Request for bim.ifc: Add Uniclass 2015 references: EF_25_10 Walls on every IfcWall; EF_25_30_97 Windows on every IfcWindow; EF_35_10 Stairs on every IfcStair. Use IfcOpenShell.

First a look at what the model holds.

```python
import ifcopenshell

model = ifcopenshell.open("bim.ifc")
print(model.schema)
print("classifications:", [c.Name for c in model.by_type("IfcClassification")])
for ifc_class in ("IfcDoor", "IfcRoof", "IfcStair", "IfcWall", "IfcWindow"):
    print(ifc_class, len(model.by_type(ifc_class)))
```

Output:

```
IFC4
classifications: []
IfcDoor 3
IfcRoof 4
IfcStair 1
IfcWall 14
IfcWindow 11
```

```python
import ifcopenshell
import ifcopenshell.api.classification

model = ifcopenshell.open("bim.ifc")

system = ifcopenshell.api.classification.add_classification(model, classification="Uniclass 2015")

codes = {
    "IfcWall": ("EF_25_10", "Walls"),
    "IfcWindow": ("EF_25_30_97", "Windows"),
    "IfcStair": ("EF_35_10", "Stairs"),
}
for ifc_class, (code, name) in codes.items():
    products = model.by_type(ifc_class)
    ifcopenshell.api.classification.add_reference(
        model, products=products, classification=system, identification=code, name=name
    )
    print(code, len(products))

model.write("bim_edited.ifc")
```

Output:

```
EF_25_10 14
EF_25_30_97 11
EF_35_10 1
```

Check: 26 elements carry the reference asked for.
